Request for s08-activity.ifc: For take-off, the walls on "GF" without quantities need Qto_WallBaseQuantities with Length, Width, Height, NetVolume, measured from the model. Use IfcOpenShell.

First a look at what the model holds.

```python
import ifcopenshell
import ifcopenshell.util.element
import ifcopenshell.util.unit

model = ifcopenshell.open("s08-activity.ifc")
print(model.schema)
for unit_type in ("LENGTHUNIT", "AREAUNIT", "VOLUMEUNIT"):
    print(unit_type, ifcopenshell.util.unit.calculate_unit_scale(model, unit_type))
storey = next(s for s in model.by_type("IfcBuildingStorey") if s.Name == "GF")
walls = [e for e in ifcopenshell.util.element.get_decomposition(storey) if e.is_a("IfcWall")]
for e in sorted(walls, key=lambda e: e.id()):
    print(e.id(), e.is_a(), e.Name, list(ifcopenshell.util.element.get_psets(e, qtos_only=True)), sep=" | ")
```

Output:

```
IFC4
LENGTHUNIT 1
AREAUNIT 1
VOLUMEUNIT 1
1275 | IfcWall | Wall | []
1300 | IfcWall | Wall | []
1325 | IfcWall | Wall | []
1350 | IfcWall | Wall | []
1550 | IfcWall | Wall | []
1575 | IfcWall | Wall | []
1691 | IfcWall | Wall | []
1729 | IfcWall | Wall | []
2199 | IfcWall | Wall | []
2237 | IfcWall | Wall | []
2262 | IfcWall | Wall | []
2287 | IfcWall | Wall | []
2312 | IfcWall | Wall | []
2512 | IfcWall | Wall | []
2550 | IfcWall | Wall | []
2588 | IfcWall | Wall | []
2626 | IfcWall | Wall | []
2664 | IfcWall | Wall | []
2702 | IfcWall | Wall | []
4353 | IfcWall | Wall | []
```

```python
import ifcopenshell
import ifcopenshell.api.pset
import ifcopenshell.geom
import ifcopenshell.util.element
import ifcopenshell.util.shape
import ifcopenshell.util.unit

model = ifcopenshell.open("s08-activity.ifc")
unit_scale = ifcopenshell.util.unit.calculate_unit_scale(model)
volume_scale = ifcopenshell.util.unit.calculate_unit_scale(model, "VOLUMEUNIT")
settings = ifcopenshell.geom.settings()

storey = next(s for s in model.by_type("IfcBuildingStorey") if s.Name == "GF")
walls = [e for e in ifcopenshell.util.element.get_decomposition(storey) if e.is_a("IfcWall")]

for e in sorted(walls, key=lambda e: e.id()):
    if ifcopenshell.util.element.get_psets(e, qtos_only=True, should_inherit=False):
        continue
    # Geometry comes back in metres, in the element's own axes.
    shape = ifcopenshell.geom.create_shape(settings, e)
    values = {
        "Length": ifcopenshell.util.shape.get_x(shape.geometry) / unit_scale,
        "Width": ifcopenshell.util.shape.get_y(shape.geometry) / unit_scale,
        "Height": ifcopenshell.util.shape.get_z(shape.geometry) / unit_scale,
        "NetVolume": ifcopenshell.util.shape.get_volume(shape.geometry) / volume_scale,
    }
    qto = ifcopenshell.api.pset.add_qto(model, product=e, name="Qto_WallBaseQuantities")
    ifcopenshell.api.pset.edit_qto(model, qto=qto, properties=values)
    print(e.id(), {k: round(v, 3) for k, v in values.items()})

model.write("s08-activity-out.ifc")
```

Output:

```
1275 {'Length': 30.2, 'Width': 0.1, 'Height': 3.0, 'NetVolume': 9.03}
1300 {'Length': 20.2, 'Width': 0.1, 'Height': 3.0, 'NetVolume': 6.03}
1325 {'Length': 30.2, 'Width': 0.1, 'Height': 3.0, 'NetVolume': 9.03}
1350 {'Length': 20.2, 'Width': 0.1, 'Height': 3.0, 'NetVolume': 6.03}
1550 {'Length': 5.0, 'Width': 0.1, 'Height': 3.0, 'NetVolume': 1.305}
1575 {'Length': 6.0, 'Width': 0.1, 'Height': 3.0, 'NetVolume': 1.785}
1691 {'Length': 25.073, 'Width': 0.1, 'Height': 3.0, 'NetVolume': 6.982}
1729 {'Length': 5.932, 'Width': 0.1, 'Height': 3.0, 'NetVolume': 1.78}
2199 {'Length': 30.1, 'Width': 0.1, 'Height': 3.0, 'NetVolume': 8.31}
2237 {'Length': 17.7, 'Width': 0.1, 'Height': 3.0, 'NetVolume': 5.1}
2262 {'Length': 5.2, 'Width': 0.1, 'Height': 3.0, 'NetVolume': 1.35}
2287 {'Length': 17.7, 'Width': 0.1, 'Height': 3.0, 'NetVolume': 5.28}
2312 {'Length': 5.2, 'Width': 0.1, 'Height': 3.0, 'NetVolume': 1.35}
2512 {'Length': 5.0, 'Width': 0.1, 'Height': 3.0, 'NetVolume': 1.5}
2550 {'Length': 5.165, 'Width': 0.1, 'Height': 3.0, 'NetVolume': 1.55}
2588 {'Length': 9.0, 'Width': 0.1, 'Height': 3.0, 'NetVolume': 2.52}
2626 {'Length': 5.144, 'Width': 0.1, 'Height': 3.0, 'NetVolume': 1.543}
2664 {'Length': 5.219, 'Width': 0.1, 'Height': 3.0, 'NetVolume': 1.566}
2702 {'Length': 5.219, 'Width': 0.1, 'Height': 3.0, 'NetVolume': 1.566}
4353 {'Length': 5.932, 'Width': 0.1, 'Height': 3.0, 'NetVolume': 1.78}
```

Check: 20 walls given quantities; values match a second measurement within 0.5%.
